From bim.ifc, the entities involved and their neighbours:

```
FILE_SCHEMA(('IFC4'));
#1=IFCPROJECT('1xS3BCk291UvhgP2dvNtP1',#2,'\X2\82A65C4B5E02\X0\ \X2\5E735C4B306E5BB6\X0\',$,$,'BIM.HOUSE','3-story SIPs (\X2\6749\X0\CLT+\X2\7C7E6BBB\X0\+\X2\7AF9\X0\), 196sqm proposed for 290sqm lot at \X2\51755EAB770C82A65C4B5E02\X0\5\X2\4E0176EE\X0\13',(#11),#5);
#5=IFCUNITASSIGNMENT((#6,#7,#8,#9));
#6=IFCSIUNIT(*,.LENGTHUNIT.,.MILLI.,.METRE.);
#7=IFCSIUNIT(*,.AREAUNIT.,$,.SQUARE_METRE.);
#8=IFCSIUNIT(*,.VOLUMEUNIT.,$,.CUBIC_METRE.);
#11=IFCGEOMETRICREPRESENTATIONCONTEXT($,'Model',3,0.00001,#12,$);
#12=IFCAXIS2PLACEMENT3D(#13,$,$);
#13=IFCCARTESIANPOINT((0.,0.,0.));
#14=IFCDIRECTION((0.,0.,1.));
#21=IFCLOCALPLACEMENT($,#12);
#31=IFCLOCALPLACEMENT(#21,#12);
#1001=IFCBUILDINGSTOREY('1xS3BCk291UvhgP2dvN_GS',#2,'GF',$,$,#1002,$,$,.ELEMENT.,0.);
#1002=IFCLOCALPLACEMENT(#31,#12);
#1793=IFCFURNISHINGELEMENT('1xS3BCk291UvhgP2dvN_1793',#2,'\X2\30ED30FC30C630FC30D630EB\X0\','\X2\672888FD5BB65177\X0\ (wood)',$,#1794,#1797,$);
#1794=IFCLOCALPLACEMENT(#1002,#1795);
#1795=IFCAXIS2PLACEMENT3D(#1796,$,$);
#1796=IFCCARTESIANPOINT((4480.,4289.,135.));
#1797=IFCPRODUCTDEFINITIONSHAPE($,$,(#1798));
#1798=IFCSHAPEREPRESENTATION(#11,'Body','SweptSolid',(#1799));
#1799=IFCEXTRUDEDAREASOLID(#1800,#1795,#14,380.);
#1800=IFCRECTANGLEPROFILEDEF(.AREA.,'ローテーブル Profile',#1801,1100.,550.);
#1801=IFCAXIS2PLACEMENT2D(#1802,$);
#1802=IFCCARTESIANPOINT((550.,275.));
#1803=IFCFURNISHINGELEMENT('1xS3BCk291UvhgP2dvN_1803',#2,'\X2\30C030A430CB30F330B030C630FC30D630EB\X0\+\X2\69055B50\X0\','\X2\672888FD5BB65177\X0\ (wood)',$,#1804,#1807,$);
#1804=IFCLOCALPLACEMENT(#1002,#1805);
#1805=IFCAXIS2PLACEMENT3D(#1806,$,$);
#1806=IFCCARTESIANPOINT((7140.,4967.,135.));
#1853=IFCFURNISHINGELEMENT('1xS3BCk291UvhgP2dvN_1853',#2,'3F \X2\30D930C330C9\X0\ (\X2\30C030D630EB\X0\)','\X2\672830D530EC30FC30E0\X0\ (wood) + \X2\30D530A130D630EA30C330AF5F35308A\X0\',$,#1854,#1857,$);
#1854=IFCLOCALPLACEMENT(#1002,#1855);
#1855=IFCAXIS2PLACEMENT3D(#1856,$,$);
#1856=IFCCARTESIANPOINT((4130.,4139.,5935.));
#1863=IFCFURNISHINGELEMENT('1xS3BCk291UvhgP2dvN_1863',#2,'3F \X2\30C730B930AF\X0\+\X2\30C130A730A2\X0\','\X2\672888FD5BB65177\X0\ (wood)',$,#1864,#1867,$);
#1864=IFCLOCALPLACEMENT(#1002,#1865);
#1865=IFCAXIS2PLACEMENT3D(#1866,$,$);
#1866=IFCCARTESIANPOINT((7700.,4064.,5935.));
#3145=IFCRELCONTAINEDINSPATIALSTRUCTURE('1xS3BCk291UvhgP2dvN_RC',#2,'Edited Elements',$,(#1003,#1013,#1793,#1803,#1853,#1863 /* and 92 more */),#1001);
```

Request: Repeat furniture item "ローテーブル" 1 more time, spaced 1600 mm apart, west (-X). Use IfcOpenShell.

```python
import numpy as np
import ifcopenshell
import ifcopenshell.api.geometry
import ifcopenshell.api.root
import ifcopenshell.util.element
import ifcopenshell.util.placement
import ifcopenshell.util.unit

model = ifcopenshell.open("bim.ifc")
unit_scale = ifcopenshell.util.unit.calculate_unit_scale(model)


def reuse_history(source, copy):
    """copy_class also copies each property set's owner history, people and application; keep the originals."""
    for rel in copy.IsDefinedBy:
        if rel.is_a("IfcRelDefinesByProperties") and (history := rel.RelatingPropertyDefinition.OwnerHistory):
            rel.RelatingPropertyDefinition.OwnerHistory = source.OwnerHistory
            ifcopenshell.util.element.remove_deep2(model, history)


source = model.by_guid("1xS3BCk291UvhgP2dvN_1793")
base = ifcopenshell.util.placement.get_local_placement(source.ObjectPlacement)
step = np.array([-1.0, 0.0, 0.0]) * 1.6 / unit_scale

for i in range(1, 2):
    copy = ifcopenshell.api.root.copy_class(model, product=source)
    copy.Representation = ifcopenshell.util.element.copy_deep(
        model, source.Representation, exclude=["IfcGeometricRepresentationContext", "IfcRepresentationMap"]
    )
    reuse_history(source, copy)
    matrix = base.copy()
    matrix[:3, 3] += i * step
    print("added at", matrix[:3, 3].round(3) + 0.0)
    ifcopenshell.api.geometry.edit_object_placement(model, product=copy, matrix=matrix, is_si=False)

model.write("bim_edited.ifc")
```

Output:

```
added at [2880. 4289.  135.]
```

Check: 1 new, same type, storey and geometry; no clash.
